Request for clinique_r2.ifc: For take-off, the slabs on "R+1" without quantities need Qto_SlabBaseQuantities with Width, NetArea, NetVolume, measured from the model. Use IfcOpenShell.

First a look at what the model holds.

```python
import ifcopenshell
import ifcopenshell.util.element
import ifcopenshell.util.unit

model = ifcopenshell.open("clinique_r2.ifc")
print(model.schema)
for unit_type in ("LENGTHUNIT", "AREAUNIT", "VOLUMEUNIT"):
    print(unit_type, ifcopenshell.util.unit.calculate_unit_scale(model, unit_type))
storey = next(s for s in model.by_type("IfcBuildingStorey") if s.Name == "R+1")
slabs = [e for e in ifcopenshell.util.element.get_decomposition(storey) if e.is_a("IfcSlab")]
for e in sorted(slabs, key=lambda e: e.id()):
    print(e.id(), e.is_a(), e.Name, list(ifcopenshell.util.element.get_psets(e, qtos_only=True)), sep=" | ")
```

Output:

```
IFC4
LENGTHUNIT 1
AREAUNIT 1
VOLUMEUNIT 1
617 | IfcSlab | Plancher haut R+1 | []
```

```python
import ifcopenshell
import ifcopenshell.api.pset
import ifcopenshell.geom
import ifcopenshell.util.element
import ifcopenshell.util.shape
import ifcopenshell.util.unit

model = ifcopenshell.open("clinique_r2.ifc")
unit_scale = ifcopenshell.util.unit.calculate_unit_scale(model)
area_scale = ifcopenshell.util.unit.calculate_unit_scale(model, "AREAUNIT")
volume_scale = ifcopenshell.util.unit.calculate_unit_scale(model, "VOLUMEUNIT")
settings = ifcopenshell.geom.settings()

storey = next(s for s in model.by_type("IfcBuildingStorey") if s.Name == "R+1")
slabs = [e for e in ifcopenshell.util.element.get_decomposition(storey) if e.is_a("IfcSlab")]

for e in sorted(slabs, key=lambda e: e.id()):
    if ifcopenshell.util.element.get_psets(e, qtos_only=True, should_inherit=False):
        continue
    # Geometry comes back in metres, in the element's own axes.
    shape = ifcopenshell.geom.create_shape(settings, e)
    values = {
        "Width": ifcopenshell.util.shape.get_z(shape.geometry) / unit_scale,
        "NetArea": ifcopenshell.util.shape.get_footprint_area(shape.geometry) / area_scale,
        "NetVolume": ifcopenshell.util.shape.get_volume(shape.geometry) / volume_scale,
    }
    qto = ifcopenshell.api.pset.add_qto(model, product=e, name="Qto_SlabBaseQuantities")
    ifcopenshell.api.pset.edit_qto(model, qto=qto, properties=values)
    print(e.id(), {k: round(v, 3) for k, v in values.items()})

model.write("clinique_r2_v2.ifc")
```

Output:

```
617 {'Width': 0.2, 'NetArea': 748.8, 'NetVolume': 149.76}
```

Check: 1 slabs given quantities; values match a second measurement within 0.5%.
